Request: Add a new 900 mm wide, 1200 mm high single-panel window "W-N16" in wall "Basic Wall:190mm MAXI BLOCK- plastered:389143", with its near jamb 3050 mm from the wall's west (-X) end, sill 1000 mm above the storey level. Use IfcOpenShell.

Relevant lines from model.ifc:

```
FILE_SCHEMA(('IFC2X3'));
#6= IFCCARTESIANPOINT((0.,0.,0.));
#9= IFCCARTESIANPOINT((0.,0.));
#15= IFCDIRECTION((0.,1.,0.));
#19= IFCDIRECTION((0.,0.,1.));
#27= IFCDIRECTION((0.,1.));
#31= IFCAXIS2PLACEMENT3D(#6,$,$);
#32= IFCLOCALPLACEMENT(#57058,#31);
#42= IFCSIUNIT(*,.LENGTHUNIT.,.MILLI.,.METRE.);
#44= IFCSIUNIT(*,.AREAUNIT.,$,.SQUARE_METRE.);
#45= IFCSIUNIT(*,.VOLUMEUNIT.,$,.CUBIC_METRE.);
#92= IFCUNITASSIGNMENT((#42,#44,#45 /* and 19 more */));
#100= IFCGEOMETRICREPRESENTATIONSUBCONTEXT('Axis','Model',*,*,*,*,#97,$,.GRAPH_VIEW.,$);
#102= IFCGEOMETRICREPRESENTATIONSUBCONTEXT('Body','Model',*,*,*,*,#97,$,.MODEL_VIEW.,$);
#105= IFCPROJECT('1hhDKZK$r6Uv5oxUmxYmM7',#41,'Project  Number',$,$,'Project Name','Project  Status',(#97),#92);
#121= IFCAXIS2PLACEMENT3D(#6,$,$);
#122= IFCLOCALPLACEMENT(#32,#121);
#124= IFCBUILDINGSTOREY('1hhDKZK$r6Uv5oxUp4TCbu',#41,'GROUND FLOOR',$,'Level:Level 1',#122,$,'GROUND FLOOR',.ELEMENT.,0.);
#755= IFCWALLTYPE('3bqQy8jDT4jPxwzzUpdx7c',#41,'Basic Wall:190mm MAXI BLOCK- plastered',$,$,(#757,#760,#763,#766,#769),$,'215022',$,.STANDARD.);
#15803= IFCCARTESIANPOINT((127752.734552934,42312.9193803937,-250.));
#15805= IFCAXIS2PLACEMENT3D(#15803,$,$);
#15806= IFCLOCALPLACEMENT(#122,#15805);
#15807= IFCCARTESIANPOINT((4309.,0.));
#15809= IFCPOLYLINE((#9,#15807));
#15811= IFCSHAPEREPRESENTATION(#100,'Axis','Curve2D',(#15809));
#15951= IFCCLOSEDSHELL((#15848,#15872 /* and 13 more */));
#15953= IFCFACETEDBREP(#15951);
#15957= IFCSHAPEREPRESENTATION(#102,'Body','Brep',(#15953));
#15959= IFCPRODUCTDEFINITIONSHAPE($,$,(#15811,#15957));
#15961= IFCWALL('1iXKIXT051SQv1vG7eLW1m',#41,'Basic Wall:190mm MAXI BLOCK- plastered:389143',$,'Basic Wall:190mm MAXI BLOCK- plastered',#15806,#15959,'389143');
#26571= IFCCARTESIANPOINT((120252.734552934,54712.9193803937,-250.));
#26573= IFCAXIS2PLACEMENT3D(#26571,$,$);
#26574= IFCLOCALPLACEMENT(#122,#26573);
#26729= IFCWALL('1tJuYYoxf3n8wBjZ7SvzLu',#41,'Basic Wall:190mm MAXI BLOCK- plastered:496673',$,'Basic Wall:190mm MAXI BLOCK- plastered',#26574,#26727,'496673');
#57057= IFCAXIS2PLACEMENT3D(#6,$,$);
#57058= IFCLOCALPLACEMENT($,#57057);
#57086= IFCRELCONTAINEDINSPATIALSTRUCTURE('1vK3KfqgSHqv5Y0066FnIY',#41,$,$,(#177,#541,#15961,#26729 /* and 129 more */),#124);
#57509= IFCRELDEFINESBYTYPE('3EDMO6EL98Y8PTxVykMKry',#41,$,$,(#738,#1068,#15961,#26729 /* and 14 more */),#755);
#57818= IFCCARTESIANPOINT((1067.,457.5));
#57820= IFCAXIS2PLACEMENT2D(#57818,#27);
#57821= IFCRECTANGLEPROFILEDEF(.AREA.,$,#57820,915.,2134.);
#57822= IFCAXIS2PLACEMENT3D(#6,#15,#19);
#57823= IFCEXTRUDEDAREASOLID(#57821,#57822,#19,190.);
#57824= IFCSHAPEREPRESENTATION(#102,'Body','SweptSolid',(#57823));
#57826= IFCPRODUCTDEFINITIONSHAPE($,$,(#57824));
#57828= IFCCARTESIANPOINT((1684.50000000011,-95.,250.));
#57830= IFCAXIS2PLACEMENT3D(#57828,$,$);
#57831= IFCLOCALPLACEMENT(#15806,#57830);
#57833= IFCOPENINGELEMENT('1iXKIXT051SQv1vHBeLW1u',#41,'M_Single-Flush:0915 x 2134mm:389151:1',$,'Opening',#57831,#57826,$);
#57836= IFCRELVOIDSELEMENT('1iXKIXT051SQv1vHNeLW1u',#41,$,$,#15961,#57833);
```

```python
import numpy as np
import ifcopenshell
import ifcopenshell.api.feature
import ifcopenshell.api.geometry
import ifcopenshell.api.root
import ifcopenshell.api.spatial
import ifcopenshell.api.type
import ifcopenshell.geom
import ifcopenshell.util.element
import ifcopenshell.util.placement
import ifcopenshell.util.representation
import ifcopenshell.util.shape
import ifcopenshell.util.unit

model = ifcopenshell.open("model.ifc")
unit_scale = ifcopenshell.util.unit.calculate_unit_scale(model)
settings = ifcopenshell.geom.settings()


def volume(element):
    """Net volume in cubic metres, openings subtracted."""
    shape = ifcopenshell.geom.create_shape(settings, element)
    return ifcopenshell.util.shape.get_volume(shape.geometry)


wall = model.by_guid("1iXKIXT051SQv1vG7eLW1m")
storey = ifcopenshell.util.element.get_container(wall, ifc_class="IfcBuildingStorey")
context = ifcopenshell.util.representation.get_context(model, "Model", "Body", "MODEL_VIEW")
before = volume(wall)

width, height, from_end, sill = 0.9, 1.2, 3.05, 1  # metres

# The wall runs along its own X axis, and the end named is its -X end.
wall_shape = ifcopenshell.geom.create_shape(settings, wall)
x, y, z = ifcopenshell.util.shape.get_vertices(wall_shape.geometry).T
start = x.min() + from_end
face, thickness = float(y.min()), float(y.max() - y.min())
wall_matrix = ifcopenshell.util.placement.get_local_placement(wall.ObjectPlacement)
level = ifcopenshell.util.placement.get_local_placement(storey.ObjectPlacement)[2, 3]


def in_wall(x, y):
    """Placement at x, y metres in the wall's axes, at sill height."""
    matrix = wall_matrix.copy()
    matrix[:, 3] = wall_matrix @ np.array([x / unit_scale, y / unit_scale, 0.0, 1.0])
    matrix[2, 3] = level + sill / unit_scale
    return matrix


# Opening: a box that overshoots both wall faces by 50 mm.
opening = ifcopenshell.api.root.create_entity(model, ifc_class="IfcOpeningElement")
box = ifcopenshell.api.geometry.add_wall_representation(
    model, context=context, length=width, height=height, thickness=thickness + 0.1
)
ifcopenshell.api.geometry.assign_representation(model, product=opening, representation=box)
ifcopenshell.api.geometry.edit_object_placement(model, product=opening, matrix=in_wall(start, face - 0.05), is_si=False)
ifcopenshell.api.feature.add_feature(model, feature=opening, element=wall)

window = ifcopenshell.api.root.create_entity(model, ifc_class="IfcWindow", name="W-N16")
window.OverallWidth, window.OverallHeight = width / unit_scale, height / unit_scale
body = ifcopenshell.api.geometry.add_window_representation(
    model,
    context=context,
    overall_width=window.OverallWidth,
    overall_height=window.OverallHeight,
    partition_type="SINGLE_PANEL",
)
ifcopenshell.api.geometry.assign_representation(model, product=window, representation=body)
ifcopenshell.api.spatial.assign_container(model, products=[window], relating_structure=storey)
fills = ifcopenshell.api.feature.add_filling(model, opening=opening, element=window)
fills.OwnerHistory = window.OwnerHistory  # required in IFC2X3

# IFC2X3 keeps the operation on the window style.
style = ifcopenshell.api.root.create_entity(model, ifc_class="IfcWindowStyle", name="W-N16")
style.OperationType, style.ConstructionType = "SINGLE_PANEL", "NOTDEFINED"
style.ParameterTakesPrecedence = style.Sizeable = False
ifcopenshell.api.type.assign_type(model, related_objects=[window], relating_type=style)

# Centre the window in the wall's thickness.
ifcopenshell.api.geometry.edit_object_placement(model, product=window, matrix=in_wall(start, face), is_si=False)
window_shape = ifcopenshell.geom.create_shape(settings, window)
depth = ifcopenshell.util.shape.get_vertices(window_shape.geometry)[:, 1]
offset = face + thickness / 2 - (depth.min() + depth.max()) / 2
ifcopenshell.api.geometry.edit_object_placement(model, product=window, matrix=in_wall(start, offset), is_si=False)

after = volume(wall)

print(f"wall volume {before:.3f} -> {after:.3f} m3")

model.write("model-out.ifc")
```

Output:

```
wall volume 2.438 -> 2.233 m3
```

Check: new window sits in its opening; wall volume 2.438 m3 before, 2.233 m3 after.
